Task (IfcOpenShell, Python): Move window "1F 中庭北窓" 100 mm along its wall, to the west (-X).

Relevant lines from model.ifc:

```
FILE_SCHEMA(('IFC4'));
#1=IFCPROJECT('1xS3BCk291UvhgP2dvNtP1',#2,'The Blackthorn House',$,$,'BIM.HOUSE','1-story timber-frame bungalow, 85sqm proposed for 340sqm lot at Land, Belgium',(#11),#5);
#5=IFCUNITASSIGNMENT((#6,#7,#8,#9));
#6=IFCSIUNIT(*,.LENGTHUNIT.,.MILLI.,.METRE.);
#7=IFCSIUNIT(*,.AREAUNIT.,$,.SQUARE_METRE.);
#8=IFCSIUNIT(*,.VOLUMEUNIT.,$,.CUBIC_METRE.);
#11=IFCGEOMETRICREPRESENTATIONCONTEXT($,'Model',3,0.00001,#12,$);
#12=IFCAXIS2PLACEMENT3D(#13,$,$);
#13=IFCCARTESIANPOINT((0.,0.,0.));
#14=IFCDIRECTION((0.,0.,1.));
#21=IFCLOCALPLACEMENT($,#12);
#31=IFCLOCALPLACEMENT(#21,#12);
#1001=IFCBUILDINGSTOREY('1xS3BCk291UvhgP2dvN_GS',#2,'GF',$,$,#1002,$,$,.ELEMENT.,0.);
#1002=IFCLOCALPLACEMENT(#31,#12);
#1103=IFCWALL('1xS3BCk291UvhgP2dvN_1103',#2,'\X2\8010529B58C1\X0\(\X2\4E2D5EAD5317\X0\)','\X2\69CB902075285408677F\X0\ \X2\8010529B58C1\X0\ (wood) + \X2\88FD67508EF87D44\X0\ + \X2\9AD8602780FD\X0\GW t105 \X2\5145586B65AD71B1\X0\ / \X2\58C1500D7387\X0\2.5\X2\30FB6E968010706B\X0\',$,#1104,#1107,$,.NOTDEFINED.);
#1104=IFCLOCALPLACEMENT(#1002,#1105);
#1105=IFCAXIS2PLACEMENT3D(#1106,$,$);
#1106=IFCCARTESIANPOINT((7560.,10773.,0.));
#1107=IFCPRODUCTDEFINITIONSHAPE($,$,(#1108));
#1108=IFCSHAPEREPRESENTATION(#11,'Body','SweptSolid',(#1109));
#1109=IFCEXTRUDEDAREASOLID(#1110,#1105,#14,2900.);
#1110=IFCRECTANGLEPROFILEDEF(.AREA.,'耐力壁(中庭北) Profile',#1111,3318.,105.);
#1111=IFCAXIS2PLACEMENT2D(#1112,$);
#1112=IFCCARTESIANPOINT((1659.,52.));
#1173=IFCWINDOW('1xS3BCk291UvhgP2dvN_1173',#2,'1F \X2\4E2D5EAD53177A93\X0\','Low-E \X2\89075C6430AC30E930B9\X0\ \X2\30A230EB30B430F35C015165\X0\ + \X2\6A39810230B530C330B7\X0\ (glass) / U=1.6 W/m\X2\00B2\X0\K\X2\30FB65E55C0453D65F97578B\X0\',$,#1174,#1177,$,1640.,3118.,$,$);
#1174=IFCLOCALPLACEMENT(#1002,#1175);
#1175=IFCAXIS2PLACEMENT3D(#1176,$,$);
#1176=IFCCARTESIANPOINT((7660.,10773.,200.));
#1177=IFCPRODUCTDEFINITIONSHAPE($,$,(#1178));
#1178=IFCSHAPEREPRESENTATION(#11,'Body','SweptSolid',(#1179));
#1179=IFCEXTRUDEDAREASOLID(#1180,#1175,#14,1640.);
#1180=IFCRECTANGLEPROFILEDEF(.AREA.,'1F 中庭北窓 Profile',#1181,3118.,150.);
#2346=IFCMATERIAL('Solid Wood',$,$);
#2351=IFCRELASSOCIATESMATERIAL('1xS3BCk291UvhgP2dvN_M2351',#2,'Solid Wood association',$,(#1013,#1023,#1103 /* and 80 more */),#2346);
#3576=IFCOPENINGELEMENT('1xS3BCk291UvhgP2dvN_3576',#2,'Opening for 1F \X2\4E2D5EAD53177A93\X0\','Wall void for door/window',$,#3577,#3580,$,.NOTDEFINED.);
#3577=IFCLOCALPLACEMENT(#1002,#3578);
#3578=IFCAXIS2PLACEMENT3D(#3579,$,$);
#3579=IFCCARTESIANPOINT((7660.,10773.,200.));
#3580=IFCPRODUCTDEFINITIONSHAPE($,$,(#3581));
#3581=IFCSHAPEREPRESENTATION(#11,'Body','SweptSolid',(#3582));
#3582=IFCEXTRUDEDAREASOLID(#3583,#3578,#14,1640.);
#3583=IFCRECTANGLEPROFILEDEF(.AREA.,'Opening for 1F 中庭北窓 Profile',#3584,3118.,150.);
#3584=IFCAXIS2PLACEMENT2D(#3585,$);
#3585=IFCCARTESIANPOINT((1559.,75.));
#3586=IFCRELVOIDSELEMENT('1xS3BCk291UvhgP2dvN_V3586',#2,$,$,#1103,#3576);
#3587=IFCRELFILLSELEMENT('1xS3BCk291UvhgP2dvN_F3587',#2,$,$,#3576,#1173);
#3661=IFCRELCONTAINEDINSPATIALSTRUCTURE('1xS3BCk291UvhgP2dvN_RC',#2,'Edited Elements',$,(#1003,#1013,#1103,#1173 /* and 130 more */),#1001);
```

```python
import ifcopenshell
import ifcopenshell.api.geometry
import ifcopenshell.util.placement

model = ifcopenshell.open("model.ifc")

window = model.by_id(1173)
opening = window.FillsVoids[0].RelatingOpeningElement
wall = opening.VoidsElements[0].RelatingBuildingElement

wall_matrix = ifcopenshell.util.placement.get_local_placement(wall.ObjectPlacement)
shift = wall_matrix[:3, 0] * -100.0
before = ifcopenshell.util.placement.get_local_placement(window.ObjectPlacement)[:3, 3].copy()

# The window is not placed relative to its opening, so move both.
for product in (opening, window):
    matrix = ifcopenshell.util.placement.get_local_placement(product.ObjectPlacement)
    matrix[:3, 3] += shift
    ifcopenshell.api.geometry.edit_object_placement(model, product=product, matrix=matrix, is_si=False)

after = ifcopenshell.util.placement.get_local_placement(window.ObjectPlacement)[:3, 3]
print("window moved by", (after - before).round(3) + 0.0)

model.write("model_edited.ifc")
```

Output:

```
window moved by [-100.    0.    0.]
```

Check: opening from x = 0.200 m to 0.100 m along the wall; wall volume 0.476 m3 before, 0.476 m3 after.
